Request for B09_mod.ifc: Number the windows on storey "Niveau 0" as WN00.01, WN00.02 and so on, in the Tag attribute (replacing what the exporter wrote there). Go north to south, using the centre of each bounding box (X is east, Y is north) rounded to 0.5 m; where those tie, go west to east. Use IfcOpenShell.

First a look at what the model holds.

```python
import ifcopenshell
import ifcopenshell.util.element
import ifcopenshell.util.placement

model = ifcopenshell.open("B09_mod.ifc")
print(model.schema)
storey = next(s for s in model.by_type("IfcBuildingStorey") if s.Name == "Niveau 0")
windows = [e for e in ifcopenshell.util.element.get_decomposition(storey) if e.is_a("IfcWindow")]
for e in sorted(windows, key=lambda e: e.id()):
    origin = ifcopenshell.util.placement.get_local_placement(e.ObjectPlacement)[:3, 3]
    print(e.id(), e.Tag, e.Name, origin.round(2) + 0.0, sep=" | ")
```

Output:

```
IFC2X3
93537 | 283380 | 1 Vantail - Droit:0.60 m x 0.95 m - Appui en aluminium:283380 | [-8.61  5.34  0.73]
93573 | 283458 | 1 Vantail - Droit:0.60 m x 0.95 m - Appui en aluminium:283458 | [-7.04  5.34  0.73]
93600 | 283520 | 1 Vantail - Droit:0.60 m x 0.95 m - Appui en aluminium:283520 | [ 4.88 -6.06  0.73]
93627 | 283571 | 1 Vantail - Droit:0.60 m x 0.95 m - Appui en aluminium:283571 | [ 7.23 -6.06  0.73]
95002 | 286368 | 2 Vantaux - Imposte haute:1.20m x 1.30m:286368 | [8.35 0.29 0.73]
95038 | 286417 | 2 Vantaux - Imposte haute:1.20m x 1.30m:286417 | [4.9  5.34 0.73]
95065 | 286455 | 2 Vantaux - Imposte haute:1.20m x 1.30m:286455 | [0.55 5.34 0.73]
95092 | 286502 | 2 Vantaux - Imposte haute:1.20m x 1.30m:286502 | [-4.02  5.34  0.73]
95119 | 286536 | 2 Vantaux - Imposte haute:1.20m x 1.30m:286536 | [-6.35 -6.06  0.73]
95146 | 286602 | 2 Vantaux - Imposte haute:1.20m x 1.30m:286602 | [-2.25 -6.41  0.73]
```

```python
import ifcopenshell
import ifcopenshell.geom
import ifcopenshell.util.element
import ifcopenshell.util.shape

model = ifcopenshell.open("B09_mod.ifc")
settings = ifcopenshell.geom.settings()
settings.set("use-world-coords", True)


def centre(element):
    shape = ifcopenshell.geom.create_shape(settings, element)
    return ifcopenshell.util.shape.get_bbox_centroid(shape.geometry)


storey = next(s for s in model.by_type("IfcBuildingStorey") if s.Name == "Niveau 0")
windows = [e for e in ifcopenshell.util.element.get_decomposition(storey) if e.is_a("IfcWindow")]

# Insertion points can sit at a corner or the storey origin, so sort by the geometry (in metres).
centres = {e: centre(e) for e in windows}
windows.sort(key=lambda e: (-round(centres[e][1] / 0.5), centres[e][0]))

for i, e in enumerate(windows, start=1):
    number = f"WN00.{i:02d}"
    e.Tag = number
    print(e.id(), number)

model.write("B09_mod-out.ifc")
```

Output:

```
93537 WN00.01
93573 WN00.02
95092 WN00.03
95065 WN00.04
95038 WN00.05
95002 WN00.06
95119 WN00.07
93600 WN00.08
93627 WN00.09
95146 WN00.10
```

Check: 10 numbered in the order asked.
